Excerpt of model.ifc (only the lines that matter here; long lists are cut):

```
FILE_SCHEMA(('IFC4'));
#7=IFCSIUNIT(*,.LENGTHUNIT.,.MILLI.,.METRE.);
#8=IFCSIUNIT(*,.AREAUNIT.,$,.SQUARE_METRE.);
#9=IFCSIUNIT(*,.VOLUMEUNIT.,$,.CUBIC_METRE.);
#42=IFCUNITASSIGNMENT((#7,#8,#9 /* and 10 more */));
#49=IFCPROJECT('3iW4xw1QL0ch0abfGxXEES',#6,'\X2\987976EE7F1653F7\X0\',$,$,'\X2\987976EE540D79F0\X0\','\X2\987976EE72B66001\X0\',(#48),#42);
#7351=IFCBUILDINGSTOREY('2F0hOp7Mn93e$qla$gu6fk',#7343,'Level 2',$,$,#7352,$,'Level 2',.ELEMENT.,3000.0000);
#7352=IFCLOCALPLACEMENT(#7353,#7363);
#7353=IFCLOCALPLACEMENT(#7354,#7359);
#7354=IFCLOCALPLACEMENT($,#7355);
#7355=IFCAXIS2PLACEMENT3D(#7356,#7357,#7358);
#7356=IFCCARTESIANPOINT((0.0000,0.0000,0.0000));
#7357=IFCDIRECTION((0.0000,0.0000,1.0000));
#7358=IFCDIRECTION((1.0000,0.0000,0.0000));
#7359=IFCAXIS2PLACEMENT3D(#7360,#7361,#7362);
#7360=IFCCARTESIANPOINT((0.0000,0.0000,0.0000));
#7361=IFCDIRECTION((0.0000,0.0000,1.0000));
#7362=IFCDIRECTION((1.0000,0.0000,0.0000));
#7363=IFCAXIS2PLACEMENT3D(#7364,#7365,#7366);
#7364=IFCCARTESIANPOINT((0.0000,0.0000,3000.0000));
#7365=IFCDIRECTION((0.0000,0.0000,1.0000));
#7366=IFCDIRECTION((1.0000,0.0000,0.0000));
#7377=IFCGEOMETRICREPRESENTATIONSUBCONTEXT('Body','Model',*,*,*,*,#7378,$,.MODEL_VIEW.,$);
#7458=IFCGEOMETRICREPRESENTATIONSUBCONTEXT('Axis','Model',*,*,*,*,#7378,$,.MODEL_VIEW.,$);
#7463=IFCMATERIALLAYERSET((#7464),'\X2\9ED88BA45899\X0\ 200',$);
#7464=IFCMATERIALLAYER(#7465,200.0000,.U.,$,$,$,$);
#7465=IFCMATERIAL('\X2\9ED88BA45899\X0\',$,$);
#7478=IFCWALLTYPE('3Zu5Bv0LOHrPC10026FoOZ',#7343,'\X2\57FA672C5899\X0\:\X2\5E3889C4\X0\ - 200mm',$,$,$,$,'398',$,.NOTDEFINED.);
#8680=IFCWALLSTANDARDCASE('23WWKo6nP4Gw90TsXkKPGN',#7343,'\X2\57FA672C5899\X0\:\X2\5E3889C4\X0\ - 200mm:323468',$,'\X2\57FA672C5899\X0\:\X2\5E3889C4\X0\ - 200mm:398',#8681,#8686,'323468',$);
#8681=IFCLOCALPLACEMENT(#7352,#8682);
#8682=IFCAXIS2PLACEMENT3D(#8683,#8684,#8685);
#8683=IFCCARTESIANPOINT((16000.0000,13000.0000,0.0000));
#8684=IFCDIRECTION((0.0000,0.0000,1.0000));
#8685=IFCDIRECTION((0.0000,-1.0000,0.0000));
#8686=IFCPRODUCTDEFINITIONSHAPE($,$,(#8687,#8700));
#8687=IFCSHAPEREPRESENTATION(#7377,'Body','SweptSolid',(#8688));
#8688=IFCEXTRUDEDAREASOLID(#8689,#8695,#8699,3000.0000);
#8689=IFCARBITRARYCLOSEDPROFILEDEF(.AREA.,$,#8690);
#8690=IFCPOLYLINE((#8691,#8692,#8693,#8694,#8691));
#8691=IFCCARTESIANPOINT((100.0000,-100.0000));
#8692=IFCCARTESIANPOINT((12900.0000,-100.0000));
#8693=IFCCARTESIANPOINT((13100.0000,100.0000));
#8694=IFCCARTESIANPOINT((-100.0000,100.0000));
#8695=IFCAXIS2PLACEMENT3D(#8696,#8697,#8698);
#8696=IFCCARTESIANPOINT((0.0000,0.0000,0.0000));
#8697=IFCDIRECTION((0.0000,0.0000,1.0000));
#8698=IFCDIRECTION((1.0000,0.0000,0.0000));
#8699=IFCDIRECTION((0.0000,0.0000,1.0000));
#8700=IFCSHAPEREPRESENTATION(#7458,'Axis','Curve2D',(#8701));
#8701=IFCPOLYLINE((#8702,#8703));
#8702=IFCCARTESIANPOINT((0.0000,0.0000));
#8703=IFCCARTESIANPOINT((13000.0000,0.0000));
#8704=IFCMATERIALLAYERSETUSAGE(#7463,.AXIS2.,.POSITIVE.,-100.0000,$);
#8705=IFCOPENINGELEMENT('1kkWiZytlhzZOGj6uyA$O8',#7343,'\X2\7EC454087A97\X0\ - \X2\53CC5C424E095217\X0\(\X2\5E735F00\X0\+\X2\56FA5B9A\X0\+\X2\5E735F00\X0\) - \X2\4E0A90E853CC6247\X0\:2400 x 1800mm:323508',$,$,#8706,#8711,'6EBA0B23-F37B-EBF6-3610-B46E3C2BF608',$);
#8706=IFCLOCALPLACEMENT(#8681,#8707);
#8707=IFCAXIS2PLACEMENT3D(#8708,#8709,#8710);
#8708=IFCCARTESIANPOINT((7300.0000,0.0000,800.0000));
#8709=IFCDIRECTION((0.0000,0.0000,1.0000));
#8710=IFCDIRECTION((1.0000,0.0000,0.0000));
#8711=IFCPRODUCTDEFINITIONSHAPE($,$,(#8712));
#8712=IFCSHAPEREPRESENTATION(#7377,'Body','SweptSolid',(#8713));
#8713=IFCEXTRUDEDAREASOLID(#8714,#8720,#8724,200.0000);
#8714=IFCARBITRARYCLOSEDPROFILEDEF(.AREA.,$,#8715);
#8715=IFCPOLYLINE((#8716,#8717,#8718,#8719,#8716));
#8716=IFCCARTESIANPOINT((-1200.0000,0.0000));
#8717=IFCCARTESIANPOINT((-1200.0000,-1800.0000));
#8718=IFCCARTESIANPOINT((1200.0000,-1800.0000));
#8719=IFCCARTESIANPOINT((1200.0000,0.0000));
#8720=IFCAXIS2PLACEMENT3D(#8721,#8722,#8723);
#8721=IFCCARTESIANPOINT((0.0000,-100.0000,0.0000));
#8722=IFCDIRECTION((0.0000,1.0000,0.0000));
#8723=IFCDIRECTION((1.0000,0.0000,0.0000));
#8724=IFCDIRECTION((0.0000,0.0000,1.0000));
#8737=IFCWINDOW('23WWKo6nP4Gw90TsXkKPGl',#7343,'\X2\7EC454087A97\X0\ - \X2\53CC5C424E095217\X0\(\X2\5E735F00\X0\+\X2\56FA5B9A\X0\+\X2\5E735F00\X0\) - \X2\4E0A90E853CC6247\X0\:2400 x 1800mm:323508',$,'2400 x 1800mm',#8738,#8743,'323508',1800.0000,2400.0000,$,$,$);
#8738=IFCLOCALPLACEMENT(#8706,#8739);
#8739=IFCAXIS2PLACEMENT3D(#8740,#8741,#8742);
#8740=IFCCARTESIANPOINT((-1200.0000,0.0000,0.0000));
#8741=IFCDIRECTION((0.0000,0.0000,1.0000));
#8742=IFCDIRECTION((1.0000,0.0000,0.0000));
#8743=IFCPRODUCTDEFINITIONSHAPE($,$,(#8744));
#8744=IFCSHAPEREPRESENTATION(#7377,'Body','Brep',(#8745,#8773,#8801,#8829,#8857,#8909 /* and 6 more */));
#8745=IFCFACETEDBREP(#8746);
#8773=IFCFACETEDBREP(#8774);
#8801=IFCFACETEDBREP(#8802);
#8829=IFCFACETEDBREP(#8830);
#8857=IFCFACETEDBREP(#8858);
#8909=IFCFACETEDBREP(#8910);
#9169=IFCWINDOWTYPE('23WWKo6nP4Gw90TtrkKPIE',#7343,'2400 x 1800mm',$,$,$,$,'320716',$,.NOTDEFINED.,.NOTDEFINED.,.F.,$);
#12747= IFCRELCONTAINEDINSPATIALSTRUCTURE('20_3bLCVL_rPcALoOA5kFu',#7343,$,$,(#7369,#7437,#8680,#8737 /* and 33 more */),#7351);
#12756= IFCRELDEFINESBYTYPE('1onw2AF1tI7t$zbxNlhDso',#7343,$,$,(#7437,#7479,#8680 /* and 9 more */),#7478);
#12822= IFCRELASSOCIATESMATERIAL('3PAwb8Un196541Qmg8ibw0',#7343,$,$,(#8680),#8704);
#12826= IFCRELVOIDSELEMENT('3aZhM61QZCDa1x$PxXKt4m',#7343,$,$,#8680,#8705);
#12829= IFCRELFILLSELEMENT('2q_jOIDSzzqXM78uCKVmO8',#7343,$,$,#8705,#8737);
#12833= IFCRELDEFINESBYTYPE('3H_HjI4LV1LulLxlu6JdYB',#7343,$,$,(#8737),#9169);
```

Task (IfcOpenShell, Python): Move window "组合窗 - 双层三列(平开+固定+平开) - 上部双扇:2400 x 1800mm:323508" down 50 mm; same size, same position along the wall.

```python
import numpy as np
import ifcopenshell
import ifcopenshell.api.geometry
import ifcopenshell.util.placement
import ifcopenshell.util.unit

model = ifcopenshell.open("model.ifc")
unit_scale = ifcopenshell.util.unit.calculate_unit_scale(model)

window = model.by_id(8737)
opening = window.FillsVoids[0].RelatingOpeningElement
dz = -50.0

shift = np.array([0.0, 0.0, dz])
# The window is placed relative to its opening, so it follows when the opening moves.
matrix = ifcopenshell.util.placement.get_local_placement(opening.ObjectPlacement)
matrix[:3, 3] += shift
ifcopenshell.api.geometry.edit_object_placement(
    model, product=opening, matrix=matrix, is_si=False, should_transform_children=True
)

print(f"moved by {dz * unit_scale:+.3f} m")

model.write("model_edited.ifc")
```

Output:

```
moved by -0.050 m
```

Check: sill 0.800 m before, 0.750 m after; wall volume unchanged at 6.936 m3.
